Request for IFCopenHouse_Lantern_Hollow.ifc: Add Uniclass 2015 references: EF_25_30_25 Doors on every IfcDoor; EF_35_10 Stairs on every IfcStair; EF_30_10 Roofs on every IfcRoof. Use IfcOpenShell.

First a look at what the model holds.

```python
import ifcopenshell

model = ifcopenshell.open("IFCopenHouse_Lantern_Hollow.ifc")
print(model.schema)
print("classifications:", [c.Name for c in model.by_type("IfcClassification")])
for ifc_class in ("IfcDoor", "IfcRoof", "IfcStair", "IfcWall", "IfcWindow"):
    print(ifc_class, len(model.by_type(ifc_class)))
```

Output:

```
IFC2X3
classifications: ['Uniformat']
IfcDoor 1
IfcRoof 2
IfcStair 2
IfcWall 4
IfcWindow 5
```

```python
import ifcopenshell
import ifcopenshell.api.classification

model = ifcopenshell.open("IFCopenHouse_Lantern_Hollow.ifc")

# IFC2X3 requires Source and Edition and has no link from the project to the system.
system = model.create_entity("IfcClassification", Source="NBS", Edition="2015", Name="Uniclass 2015")

codes = {
    "IfcDoor": ("EF_25_30_25", "Doors"),
    "IfcStair": ("EF_35_10", "Stairs"),
    "IfcRoof": ("EF_30_10", "Roofs"),
}
for ifc_class, (code, name) in codes.items():
    products = model.by_type(ifc_class)
    ifcopenshell.api.classification.add_reference(
        model, products=products, classification=system, identification=code, name=name
    )
    print(code, len(products))

model.write("IFCopenHouse_Lantern_Hollow_updated.ifc")
```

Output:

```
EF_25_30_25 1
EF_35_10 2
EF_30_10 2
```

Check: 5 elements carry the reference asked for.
